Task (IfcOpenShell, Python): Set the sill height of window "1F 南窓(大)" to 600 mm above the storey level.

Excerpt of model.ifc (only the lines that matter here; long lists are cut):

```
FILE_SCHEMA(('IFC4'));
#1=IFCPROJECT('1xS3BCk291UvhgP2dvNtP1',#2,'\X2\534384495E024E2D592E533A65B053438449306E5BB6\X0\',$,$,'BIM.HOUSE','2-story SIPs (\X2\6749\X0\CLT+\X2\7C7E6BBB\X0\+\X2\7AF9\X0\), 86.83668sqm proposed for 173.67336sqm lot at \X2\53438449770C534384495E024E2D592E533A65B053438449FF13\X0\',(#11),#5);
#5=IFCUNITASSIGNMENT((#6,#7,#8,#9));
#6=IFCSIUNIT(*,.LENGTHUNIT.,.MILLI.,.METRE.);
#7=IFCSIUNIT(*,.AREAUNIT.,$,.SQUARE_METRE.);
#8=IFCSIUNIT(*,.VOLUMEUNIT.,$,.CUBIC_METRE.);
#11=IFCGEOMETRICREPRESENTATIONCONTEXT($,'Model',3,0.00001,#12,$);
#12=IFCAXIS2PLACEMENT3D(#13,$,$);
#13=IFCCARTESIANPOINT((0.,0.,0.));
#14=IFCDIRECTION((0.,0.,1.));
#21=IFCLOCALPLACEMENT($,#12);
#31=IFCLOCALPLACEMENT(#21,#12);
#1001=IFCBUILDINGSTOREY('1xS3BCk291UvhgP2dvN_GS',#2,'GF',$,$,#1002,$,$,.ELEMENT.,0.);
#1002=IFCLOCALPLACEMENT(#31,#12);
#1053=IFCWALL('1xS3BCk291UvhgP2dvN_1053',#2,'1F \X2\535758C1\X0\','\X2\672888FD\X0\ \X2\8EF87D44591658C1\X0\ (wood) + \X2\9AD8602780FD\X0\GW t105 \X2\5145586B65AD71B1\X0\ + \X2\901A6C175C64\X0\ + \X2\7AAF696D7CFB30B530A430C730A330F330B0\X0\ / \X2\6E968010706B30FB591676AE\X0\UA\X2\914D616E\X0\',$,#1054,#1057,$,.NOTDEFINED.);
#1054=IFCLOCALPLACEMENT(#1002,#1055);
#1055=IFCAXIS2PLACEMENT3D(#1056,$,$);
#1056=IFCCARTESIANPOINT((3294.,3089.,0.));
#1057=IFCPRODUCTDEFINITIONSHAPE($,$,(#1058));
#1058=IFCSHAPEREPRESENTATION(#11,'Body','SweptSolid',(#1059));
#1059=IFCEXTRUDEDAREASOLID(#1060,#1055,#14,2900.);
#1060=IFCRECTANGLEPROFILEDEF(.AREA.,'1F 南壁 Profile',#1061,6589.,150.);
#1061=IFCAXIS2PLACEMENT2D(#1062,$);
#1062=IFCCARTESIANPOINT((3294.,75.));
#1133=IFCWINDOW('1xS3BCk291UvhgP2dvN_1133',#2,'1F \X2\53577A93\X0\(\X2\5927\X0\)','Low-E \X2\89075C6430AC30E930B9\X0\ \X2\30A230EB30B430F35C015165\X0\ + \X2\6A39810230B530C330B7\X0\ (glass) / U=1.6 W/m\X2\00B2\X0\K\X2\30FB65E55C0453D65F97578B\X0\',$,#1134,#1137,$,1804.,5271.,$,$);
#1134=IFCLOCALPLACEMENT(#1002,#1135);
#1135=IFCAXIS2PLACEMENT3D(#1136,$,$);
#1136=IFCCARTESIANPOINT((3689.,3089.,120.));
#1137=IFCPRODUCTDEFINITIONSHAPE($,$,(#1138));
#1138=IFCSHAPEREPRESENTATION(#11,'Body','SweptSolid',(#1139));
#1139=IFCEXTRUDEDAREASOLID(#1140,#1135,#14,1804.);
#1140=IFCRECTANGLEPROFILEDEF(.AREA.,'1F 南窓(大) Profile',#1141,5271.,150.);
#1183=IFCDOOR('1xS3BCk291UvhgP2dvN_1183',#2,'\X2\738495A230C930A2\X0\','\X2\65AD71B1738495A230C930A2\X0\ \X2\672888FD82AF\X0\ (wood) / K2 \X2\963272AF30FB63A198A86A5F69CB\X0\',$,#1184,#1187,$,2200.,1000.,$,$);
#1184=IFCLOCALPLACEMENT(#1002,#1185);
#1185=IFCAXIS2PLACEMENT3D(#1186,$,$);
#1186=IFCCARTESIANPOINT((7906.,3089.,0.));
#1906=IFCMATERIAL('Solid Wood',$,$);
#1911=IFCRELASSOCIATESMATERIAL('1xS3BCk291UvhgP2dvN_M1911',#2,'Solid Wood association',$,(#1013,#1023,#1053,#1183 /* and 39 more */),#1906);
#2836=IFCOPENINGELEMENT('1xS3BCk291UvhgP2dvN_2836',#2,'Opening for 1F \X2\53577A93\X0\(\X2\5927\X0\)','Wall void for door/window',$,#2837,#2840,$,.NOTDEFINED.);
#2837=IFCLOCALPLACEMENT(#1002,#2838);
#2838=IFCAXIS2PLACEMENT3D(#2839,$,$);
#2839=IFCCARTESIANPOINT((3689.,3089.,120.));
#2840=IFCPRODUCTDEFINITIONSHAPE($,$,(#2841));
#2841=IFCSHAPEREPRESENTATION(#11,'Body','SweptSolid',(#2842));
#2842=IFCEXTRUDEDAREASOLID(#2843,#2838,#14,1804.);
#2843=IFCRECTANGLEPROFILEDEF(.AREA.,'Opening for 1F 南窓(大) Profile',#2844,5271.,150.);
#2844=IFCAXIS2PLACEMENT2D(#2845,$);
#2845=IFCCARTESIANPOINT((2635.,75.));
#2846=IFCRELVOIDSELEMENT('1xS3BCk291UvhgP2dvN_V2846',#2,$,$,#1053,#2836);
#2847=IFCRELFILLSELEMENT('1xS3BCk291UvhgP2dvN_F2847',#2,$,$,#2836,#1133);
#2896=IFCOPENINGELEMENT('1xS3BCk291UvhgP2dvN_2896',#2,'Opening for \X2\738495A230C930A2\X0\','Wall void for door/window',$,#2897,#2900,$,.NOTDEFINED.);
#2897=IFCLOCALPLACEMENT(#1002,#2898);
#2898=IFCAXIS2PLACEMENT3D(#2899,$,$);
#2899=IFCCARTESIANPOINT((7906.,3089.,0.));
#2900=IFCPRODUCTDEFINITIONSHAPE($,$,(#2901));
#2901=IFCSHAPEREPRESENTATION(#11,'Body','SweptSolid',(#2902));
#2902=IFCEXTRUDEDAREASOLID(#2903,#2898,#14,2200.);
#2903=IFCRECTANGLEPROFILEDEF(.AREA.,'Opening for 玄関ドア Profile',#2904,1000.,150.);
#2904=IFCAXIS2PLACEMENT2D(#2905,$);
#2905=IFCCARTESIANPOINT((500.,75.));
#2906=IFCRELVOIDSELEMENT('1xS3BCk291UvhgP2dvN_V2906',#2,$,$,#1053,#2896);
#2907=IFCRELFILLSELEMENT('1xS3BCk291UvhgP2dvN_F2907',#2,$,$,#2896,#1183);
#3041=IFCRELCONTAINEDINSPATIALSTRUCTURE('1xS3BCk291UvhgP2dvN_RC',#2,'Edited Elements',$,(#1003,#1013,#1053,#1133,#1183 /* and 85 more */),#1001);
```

```python
import numpy as np
import ifcopenshell
import ifcopenshell.api.geometry
import ifcopenshell.geom
import ifcopenshell.util.element
import ifcopenshell.util.placement
import ifcopenshell.util.shape
import ifcopenshell.util.unit

model = ifcopenshell.open("model.ifc")
unit_scale = ifcopenshell.util.unit.calculate_unit_scale(model)

window = model.by_id(1133)
opening = window.FillsVoids[0].RelatingOpeningElement
storey = ifcopenshell.util.element.get_container(window, ifc_class="IfcBuildingStorey")
level = ifcopenshell.util.placement.get_local_placement(storey.ObjectPlacement)[2, 3]

# The opening's origin need not be at the sill, so measure its lowest point.
shape = ifcopenshell.geom.create_shape(ifcopenshell.geom.settings(), opening)
bottom = ifcopenshell.util.shape.get_shape_bottom_elevation(shape, shape.geometry) / unit_scale
dz = level + 600.0 - bottom

shift = np.array([0.0, 0.0, dz])
# The window is not placed relative to its opening, so move both.
for product in (opening, window):
    matrix = ifcopenshell.util.placement.get_local_placement(product.ObjectPlacement)
    matrix[:3, 3] += shift
    ifcopenshell.api.geometry.edit_object_placement(model, product=product, matrix=matrix, is_si=False)

print(f"moved by {dz * unit_scale:+.3f} m")

model.write("model_updated.ifc")
```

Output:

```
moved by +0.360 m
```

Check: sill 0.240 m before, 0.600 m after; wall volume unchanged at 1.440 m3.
